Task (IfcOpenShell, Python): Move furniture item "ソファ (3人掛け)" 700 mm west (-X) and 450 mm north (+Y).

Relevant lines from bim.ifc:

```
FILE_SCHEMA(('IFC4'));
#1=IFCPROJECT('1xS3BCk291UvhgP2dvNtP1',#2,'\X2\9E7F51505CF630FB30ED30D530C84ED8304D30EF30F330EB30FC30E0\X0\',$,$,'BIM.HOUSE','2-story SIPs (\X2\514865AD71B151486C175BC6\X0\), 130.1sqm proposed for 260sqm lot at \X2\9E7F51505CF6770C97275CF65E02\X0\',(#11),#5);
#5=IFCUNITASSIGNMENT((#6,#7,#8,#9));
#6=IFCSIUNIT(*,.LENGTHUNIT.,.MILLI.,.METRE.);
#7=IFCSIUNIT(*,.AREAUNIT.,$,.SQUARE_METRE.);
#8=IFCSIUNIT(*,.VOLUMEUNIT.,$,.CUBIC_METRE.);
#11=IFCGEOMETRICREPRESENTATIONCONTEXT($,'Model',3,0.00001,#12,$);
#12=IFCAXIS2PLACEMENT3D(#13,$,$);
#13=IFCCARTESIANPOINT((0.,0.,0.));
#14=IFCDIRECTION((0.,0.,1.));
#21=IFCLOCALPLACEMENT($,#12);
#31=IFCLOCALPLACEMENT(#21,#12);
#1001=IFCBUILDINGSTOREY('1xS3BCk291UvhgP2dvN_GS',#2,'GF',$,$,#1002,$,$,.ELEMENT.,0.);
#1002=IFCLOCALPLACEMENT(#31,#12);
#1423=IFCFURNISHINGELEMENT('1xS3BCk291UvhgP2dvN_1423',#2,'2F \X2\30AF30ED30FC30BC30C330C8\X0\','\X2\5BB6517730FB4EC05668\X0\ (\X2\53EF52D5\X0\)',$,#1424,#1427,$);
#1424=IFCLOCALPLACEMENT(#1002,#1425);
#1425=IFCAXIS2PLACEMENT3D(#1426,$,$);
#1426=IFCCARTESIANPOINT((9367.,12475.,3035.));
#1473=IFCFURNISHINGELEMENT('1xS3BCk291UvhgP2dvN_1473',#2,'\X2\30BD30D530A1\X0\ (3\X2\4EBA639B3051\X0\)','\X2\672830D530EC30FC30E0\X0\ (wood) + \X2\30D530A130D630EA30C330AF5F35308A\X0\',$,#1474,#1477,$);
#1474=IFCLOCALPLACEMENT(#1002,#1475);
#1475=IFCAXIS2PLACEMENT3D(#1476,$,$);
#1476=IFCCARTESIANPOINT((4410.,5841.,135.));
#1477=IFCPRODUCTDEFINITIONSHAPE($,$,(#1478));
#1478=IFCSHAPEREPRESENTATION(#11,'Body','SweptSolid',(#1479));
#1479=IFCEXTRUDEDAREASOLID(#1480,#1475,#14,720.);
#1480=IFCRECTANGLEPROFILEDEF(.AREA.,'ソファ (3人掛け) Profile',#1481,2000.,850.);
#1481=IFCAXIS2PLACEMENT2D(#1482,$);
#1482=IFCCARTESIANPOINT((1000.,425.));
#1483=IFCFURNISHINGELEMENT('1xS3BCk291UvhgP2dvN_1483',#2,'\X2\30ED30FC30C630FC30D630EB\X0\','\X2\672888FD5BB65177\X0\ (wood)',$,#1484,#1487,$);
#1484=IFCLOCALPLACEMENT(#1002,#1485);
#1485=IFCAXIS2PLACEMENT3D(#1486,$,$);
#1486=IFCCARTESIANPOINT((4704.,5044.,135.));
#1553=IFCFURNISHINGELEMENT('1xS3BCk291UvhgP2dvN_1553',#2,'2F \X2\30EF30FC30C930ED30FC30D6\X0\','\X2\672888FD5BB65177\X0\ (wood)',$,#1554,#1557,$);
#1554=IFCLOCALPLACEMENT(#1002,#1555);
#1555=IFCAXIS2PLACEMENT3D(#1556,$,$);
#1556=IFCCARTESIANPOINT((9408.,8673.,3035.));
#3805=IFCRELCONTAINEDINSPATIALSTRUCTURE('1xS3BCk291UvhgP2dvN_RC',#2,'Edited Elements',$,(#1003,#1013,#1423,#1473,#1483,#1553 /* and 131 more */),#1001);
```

```python
import ifcopenshell
import ifcopenshell.api.geometry
import ifcopenshell.util.placement

model = ifcopenshell.open("bim.ifc")

item = model.by_guid("1xS3BCk291UvhgP2dvN_1473")
matrix = ifcopenshell.util.placement.get_local_placement(item.ObjectPlacement)
matrix[0, 3] -= 700.0
matrix[1, 3] += 450.0
ifcopenshell.api.geometry.edit_object_placement(model, product=item, matrix=matrix, is_si=False)

print(ifcopenshell.util.placement.get_local_placement(item.ObjectPlacement).round(3) + 0.0)

model.write("bim_v2.ifc")
```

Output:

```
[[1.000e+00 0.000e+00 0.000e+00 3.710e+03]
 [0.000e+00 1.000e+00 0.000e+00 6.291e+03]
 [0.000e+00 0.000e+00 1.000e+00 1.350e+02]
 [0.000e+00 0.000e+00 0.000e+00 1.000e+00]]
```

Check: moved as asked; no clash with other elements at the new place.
